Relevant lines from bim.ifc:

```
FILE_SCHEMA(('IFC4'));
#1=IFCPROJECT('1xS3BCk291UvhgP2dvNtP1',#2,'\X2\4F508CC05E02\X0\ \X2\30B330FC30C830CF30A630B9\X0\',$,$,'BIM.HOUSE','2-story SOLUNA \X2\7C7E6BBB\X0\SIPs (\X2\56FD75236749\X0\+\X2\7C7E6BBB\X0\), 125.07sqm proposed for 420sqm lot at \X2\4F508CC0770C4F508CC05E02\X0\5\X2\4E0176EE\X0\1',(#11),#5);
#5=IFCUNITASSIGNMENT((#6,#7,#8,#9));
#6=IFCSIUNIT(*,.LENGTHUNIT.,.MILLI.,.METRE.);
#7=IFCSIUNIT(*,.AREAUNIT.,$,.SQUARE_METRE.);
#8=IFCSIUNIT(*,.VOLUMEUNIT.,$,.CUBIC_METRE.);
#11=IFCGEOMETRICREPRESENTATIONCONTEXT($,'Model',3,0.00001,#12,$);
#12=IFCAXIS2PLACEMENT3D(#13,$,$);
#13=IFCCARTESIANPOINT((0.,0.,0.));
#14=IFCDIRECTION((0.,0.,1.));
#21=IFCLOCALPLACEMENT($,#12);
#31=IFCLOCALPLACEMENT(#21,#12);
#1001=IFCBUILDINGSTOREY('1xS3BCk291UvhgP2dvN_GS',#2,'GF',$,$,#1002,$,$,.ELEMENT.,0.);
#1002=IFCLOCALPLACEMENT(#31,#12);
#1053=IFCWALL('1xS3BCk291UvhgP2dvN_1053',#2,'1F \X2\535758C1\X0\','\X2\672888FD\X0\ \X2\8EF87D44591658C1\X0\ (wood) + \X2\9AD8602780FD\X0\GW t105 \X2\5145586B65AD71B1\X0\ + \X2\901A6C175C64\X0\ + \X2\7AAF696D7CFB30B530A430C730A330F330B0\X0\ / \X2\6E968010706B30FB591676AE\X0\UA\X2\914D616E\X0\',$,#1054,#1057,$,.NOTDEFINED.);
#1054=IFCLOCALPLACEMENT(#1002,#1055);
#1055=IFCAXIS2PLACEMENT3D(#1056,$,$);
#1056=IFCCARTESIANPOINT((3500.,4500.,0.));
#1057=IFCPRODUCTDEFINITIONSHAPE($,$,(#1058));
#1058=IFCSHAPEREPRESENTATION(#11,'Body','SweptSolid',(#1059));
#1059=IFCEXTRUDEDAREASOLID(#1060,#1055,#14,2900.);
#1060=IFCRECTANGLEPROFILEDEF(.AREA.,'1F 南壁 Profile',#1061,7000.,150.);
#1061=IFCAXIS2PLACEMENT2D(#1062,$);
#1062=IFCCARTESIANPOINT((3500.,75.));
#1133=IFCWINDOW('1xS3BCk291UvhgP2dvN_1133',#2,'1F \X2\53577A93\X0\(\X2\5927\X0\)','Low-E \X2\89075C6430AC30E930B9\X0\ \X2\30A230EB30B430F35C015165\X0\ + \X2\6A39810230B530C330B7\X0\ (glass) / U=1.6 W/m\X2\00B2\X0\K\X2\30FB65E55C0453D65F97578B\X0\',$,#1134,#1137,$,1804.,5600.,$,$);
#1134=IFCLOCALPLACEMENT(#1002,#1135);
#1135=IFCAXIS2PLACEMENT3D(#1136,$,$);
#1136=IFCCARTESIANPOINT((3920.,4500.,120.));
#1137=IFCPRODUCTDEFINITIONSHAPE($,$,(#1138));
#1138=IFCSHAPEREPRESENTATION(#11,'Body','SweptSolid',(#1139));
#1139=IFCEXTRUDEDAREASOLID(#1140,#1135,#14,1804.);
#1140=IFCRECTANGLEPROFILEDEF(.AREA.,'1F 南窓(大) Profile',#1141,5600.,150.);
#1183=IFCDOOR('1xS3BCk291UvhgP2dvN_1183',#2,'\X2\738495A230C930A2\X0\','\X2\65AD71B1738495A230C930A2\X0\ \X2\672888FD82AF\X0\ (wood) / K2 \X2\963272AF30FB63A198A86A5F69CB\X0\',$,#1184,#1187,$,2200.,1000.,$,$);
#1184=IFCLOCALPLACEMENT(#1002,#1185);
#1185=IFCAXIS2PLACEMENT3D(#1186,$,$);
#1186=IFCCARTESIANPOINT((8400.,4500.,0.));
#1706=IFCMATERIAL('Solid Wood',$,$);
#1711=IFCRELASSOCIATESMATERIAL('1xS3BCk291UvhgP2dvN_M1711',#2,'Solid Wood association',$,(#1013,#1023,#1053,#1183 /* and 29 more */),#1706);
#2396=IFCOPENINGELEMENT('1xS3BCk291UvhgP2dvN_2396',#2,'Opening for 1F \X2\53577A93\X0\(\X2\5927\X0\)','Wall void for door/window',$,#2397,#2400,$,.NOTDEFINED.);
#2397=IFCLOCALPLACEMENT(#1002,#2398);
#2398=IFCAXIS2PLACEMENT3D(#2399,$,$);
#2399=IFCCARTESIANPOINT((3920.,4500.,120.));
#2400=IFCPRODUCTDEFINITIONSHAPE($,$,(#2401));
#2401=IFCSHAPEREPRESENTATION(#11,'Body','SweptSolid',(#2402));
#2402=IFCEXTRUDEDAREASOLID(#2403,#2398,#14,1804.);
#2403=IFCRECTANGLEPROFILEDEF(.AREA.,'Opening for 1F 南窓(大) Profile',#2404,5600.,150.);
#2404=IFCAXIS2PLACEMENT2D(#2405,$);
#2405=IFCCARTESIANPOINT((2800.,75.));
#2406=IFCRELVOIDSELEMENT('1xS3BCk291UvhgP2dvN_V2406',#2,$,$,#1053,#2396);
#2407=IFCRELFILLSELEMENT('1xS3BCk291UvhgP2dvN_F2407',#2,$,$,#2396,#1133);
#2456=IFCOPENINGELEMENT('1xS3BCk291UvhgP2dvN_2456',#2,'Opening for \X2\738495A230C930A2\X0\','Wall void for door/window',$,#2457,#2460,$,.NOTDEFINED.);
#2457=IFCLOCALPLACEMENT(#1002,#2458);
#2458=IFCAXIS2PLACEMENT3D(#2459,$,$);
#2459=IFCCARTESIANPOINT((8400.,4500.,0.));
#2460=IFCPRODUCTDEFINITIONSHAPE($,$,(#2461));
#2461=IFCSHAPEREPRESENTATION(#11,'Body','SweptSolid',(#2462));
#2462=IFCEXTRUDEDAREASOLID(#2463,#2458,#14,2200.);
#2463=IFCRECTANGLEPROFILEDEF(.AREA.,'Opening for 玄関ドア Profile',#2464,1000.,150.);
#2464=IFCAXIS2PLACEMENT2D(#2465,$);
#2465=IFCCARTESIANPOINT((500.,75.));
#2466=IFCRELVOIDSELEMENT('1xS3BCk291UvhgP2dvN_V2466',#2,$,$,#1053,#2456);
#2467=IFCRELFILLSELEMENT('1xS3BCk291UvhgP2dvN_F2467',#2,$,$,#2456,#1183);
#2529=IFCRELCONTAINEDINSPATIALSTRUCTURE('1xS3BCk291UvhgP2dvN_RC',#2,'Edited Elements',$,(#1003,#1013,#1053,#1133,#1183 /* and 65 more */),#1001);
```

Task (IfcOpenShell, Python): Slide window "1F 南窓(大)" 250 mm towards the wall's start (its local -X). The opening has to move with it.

```python
import ifcopenshell
import ifcopenshell.api.geometry
import ifcopenshell.util.placement

model = ifcopenshell.open("bim.ifc")

window = model.by_guid("1xS3BCk291UvhgP2dvN_1133")
opening = window.FillsVoids[0].RelatingOpeningElement
wall = opening.VoidsElements[0].RelatingBuildingElement

wall_matrix = ifcopenshell.util.placement.get_local_placement(wall.ObjectPlacement)
shift = wall_matrix[:3, 0] * -250.0
before = ifcopenshell.util.placement.get_local_placement(window.ObjectPlacement)[:3, 3].copy()

# The window is not placed relative to its opening, so move both.
for product in (opening, window):
    matrix = ifcopenshell.util.placement.get_local_placement(product.ObjectPlacement)
    matrix[:3, 3] += shift
    ifcopenshell.api.geometry.edit_object_placement(model, product=product, matrix=matrix, is_si=False)

after = ifcopenshell.util.placement.get_local_placement(window.ObjectPlacement)[:3, 3]
print("window moved by", (after - before).round(3) + 0.0)

model.write("bim-out.ifc")
```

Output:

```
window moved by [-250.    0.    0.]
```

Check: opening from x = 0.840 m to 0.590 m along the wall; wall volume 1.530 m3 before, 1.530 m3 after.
